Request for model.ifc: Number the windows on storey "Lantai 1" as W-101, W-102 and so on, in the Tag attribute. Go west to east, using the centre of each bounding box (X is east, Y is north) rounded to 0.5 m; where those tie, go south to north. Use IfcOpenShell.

First a look at what the model holds.

```python
import ifcopenshell
import ifcopenshell.util.element
import ifcopenshell.util.placement

model = ifcopenshell.open("model.ifc")
print(model.schema)
storey = next(s for s in model.by_type("IfcBuildingStorey") if s.Name == "Lantai 1")
windows = [e for e in ifcopenshell.util.element.get_decomposition(storey) if e.is_a("IfcWindow")]
for e in sorted(windows, key=lambda e: e.id()):
    origin = ifcopenshell.util.placement.get_local_placement(e.ObjectPlacement)[:3, 3]
    print(e.id(), e.Tag, e.Name, origin.round(2) + 0.0, sep=" | ")
```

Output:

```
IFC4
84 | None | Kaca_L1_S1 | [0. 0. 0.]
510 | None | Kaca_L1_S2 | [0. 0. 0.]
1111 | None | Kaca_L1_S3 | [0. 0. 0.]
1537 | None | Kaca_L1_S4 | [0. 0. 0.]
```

```python
import ifcopenshell
import ifcopenshell.geom
import ifcopenshell.util.element
import ifcopenshell.util.shape

model = ifcopenshell.open("model.ifc")
settings = ifcopenshell.geom.settings()
settings.set("use-world-coords", True)


def centre(element):
    shape = ifcopenshell.geom.create_shape(settings, element)
    return ifcopenshell.util.shape.get_bbox_centroid(shape.geometry)


storey = next(s for s in model.by_type("IfcBuildingStorey") if s.Name == "Lantai 1")
windows = [e for e in ifcopenshell.util.element.get_decomposition(storey) if e.is_a("IfcWindow")]

# Insertion points can sit at a corner or the storey origin, so sort by the geometry (in metres).
centres = {e: centre(e) for e in windows}
windows.sort(key=lambda e: (round(centres[e][0] / 0.5), centres[e][1]))

for i, e in enumerate(windows, start=1):
    number = f"W-1{i:02d}"
    e.Tag = number
    print(e.id(), number)

model.write("model-out.ifc")
```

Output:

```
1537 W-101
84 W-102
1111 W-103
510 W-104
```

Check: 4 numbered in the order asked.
